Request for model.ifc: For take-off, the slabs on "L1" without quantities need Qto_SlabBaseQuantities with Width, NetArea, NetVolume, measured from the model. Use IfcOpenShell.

First a look at what the model holds.

```python
import ifcopenshell
import ifcopenshell.util.element
import ifcopenshell.util.unit

model = ifcopenshell.open("model.ifc")
print(model.schema)
for unit_type in ("LENGTHUNIT", "AREAUNIT", "VOLUMEUNIT"):
    print(unit_type, ifcopenshell.util.unit.calculate_unit_scale(model, unit_type))
storey = next(s for s in model.by_type("IfcBuildingStorey") if s.Name == "L1")
slabs = [e for e in ifcopenshell.util.element.get_decomposition(storey) if e.is_a("IfcSlab")]
for e in sorted(slabs, key=lambda e: e.id()):
    print(e.id(), e.is_a(), e.Name, list(ifcopenshell.util.element.get_psets(e, qtos_only=True)), sep=" | ")
```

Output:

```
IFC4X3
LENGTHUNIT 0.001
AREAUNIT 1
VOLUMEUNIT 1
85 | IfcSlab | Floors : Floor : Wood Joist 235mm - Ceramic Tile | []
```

```python
import ifcopenshell
import ifcopenshell.api.pset
import ifcopenshell.geom
import ifcopenshell.util.element
import ifcopenshell.util.shape
import ifcopenshell.util.unit

model = ifcopenshell.open("model.ifc")
unit_scale = ifcopenshell.util.unit.calculate_unit_scale(model)
area_scale = ifcopenshell.util.unit.calculate_unit_scale(model, "AREAUNIT")
volume_scale = ifcopenshell.util.unit.calculate_unit_scale(model, "VOLUMEUNIT")
settings = ifcopenshell.geom.settings()

storey = next(s for s in model.by_type("IfcBuildingStorey") if s.Name == "L1")
slabs = [e for e in ifcopenshell.util.element.get_decomposition(storey) if e.is_a("IfcSlab")]

for e in sorted(slabs, key=lambda e: e.id()):
    if ifcopenshell.util.element.get_psets(e, qtos_only=True, should_inherit=False):
        continue
    # Geometry comes back in metres, in the element's own axes.
    shape = ifcopenshell.geom.create_shape(settings, e)
    values = {
        "Width": ifcopenshell.util.shape.get_z(shape.geometry) / unit_scale,
        "NetArea": ifcopenshell.util.shape.get_footprint_area(shape.geometry) / area_scale,
        "NetVolume": ifcopenshell.util.shape.get_volume(shape.geometry) / volume_scale,
    }
    qto = ifcopenshell.api.pset.add_qto(model, product=e, name="Qto_SlabBaseQuantities")
    ifcopenshell.api.pset.edit_qto(model, qto=qto, properties=values)
    print(e.id(), {k: round(v, 3) for k, v in values.items()})

model.write("model_updated.ifc")
```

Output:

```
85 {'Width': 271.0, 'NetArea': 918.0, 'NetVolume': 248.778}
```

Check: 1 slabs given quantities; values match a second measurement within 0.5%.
